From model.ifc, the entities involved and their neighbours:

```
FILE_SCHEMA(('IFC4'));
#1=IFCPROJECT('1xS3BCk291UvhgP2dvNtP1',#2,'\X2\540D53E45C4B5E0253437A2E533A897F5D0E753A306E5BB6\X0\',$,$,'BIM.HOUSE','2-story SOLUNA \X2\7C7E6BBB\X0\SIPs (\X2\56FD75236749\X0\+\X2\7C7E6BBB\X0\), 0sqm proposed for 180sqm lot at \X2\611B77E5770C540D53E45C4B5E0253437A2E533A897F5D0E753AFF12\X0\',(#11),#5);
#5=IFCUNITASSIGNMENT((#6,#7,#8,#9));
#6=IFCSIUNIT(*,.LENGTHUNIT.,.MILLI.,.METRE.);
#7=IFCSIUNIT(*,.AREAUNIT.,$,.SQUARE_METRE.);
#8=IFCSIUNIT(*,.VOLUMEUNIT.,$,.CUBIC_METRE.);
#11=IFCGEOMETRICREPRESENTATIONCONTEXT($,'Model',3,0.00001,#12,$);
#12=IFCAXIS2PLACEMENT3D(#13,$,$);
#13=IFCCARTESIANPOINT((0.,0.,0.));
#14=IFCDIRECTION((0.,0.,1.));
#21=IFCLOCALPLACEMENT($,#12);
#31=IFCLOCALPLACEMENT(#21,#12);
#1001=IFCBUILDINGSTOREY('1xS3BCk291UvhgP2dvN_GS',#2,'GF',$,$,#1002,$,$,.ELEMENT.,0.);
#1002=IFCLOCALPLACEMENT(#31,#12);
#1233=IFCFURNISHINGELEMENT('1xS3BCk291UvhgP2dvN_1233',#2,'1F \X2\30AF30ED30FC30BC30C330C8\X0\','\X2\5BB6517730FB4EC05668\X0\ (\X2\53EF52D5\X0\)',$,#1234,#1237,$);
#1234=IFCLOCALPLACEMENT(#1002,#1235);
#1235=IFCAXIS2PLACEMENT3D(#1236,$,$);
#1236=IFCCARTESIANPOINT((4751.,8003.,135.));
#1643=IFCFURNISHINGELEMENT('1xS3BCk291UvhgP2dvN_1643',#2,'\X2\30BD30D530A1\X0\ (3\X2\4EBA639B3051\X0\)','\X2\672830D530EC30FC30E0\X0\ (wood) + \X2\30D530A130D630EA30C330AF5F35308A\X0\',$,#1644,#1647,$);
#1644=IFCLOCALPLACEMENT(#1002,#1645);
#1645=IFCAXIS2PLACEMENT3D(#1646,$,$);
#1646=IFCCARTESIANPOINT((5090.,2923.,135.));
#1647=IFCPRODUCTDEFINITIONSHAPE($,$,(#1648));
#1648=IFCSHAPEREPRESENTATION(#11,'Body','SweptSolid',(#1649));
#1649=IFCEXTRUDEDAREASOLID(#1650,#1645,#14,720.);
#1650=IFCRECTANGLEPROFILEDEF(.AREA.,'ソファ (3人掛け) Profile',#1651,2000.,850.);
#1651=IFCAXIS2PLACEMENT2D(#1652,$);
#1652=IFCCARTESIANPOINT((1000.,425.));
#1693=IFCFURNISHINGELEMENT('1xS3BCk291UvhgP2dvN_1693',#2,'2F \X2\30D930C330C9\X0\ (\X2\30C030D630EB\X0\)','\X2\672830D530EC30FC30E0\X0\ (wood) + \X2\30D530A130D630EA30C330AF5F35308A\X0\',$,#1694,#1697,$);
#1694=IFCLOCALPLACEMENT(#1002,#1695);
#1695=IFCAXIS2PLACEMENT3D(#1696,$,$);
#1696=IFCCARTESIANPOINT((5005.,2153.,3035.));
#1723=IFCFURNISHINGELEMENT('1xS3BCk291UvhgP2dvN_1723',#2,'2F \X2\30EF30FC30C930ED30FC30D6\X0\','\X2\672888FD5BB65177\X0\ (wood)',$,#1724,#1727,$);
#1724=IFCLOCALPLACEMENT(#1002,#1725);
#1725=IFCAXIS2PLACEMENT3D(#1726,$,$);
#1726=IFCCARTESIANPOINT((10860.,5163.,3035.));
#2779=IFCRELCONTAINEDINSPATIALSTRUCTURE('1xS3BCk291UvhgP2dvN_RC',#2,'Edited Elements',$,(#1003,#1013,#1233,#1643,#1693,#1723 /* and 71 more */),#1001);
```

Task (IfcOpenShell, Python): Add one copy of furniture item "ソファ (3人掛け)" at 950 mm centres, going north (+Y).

```python
import numpy as np
import ifcopenshell
import ifcopenshell.api.geometry
import ifcopenshell.api.root
import ifcopenshell.util.element
import ifcopenshell.util.placement

model = ifcopenshell.open("model.ifc")


def reuse_history(source, copy):
    """copy_class also copies each property set's owner history, people and application; keep the originals."""
    for rel in copy.IsDefinedBy:
        if rel.is_a("IfcRelDefinesByProperties") and (history := rel.RelatingPropertyDefinition.OwnerHistory):
            rel.RelatingPropertyDefinition.OwnerHistory = source.OwnerHistory
            ifcopenshell.util.element.remove_deep2(model, history)


source = model.by_guid("1xS3BCk291UvhgP2dvN_1643")
base = ifcopenshell.util.placement.get_local_placement(source.ObjectPlacement)
step = np.array([0.0, 1.0, 0.0]) * 950.0

for i in range(1, 2):
    copy = ifcopenshell.api.root.copy_class(model, product=source)
    copy.Representation = ifcopenshell.util.element.copy_deep(
        model, source.Representation, exclude=["IfcGeometricRepresentationContext", "IfcRepresentationMap"]
    )
    reuse_history(source, copy)
    matrix = base.copy()
    matrix[:3, 3] += i * step
    print("added at", matrix[:3, 3].round(3) + 0.0)
    ifcopenshell.api.geometry.edit_object_placement(model, product=copy, matrix=matrix, is_si=False)

model.write("model_edited.ifc")
```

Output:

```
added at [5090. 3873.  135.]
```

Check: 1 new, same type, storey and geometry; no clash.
